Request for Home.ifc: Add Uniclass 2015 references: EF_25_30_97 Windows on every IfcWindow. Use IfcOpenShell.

First a look at what the model holds.

```python
import ifcopenshell

model = ifcopenshell.open("Home.ifc")
print(model.schema)
print("classifications:", [c.Name for c in model.by_type("IfcClassification")])
for ifc_class in ("IfcDoor", "IfcRoof", "IfcStair", "IfcWall", "IfcWindow"):
    print(ifc_class, len(model.by_type(ifc_class)))
```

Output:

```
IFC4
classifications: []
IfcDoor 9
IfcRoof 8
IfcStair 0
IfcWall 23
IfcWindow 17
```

```python
import ifcopenshell
import ifcopenshell.api.classification

model = ifcopenshell.open("Home.ifc")

system = ifcopenshell.api.classification.add_classification(model, classification="Uniclass 2015")

codes = {
    "IfcWindow": ("EF_25_30_97", "Windows"),
}
for ifc_class, (code, name) in codes.items():
    products = model.by_type(ifc_class)
    ifcopenshell.api.classification.add_reference(
        model, products=products, classification=system, identification=code, name=name
    )
    print(code, len(products))

model.write("Home_rev.ifc")
```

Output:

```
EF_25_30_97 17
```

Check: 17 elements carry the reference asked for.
